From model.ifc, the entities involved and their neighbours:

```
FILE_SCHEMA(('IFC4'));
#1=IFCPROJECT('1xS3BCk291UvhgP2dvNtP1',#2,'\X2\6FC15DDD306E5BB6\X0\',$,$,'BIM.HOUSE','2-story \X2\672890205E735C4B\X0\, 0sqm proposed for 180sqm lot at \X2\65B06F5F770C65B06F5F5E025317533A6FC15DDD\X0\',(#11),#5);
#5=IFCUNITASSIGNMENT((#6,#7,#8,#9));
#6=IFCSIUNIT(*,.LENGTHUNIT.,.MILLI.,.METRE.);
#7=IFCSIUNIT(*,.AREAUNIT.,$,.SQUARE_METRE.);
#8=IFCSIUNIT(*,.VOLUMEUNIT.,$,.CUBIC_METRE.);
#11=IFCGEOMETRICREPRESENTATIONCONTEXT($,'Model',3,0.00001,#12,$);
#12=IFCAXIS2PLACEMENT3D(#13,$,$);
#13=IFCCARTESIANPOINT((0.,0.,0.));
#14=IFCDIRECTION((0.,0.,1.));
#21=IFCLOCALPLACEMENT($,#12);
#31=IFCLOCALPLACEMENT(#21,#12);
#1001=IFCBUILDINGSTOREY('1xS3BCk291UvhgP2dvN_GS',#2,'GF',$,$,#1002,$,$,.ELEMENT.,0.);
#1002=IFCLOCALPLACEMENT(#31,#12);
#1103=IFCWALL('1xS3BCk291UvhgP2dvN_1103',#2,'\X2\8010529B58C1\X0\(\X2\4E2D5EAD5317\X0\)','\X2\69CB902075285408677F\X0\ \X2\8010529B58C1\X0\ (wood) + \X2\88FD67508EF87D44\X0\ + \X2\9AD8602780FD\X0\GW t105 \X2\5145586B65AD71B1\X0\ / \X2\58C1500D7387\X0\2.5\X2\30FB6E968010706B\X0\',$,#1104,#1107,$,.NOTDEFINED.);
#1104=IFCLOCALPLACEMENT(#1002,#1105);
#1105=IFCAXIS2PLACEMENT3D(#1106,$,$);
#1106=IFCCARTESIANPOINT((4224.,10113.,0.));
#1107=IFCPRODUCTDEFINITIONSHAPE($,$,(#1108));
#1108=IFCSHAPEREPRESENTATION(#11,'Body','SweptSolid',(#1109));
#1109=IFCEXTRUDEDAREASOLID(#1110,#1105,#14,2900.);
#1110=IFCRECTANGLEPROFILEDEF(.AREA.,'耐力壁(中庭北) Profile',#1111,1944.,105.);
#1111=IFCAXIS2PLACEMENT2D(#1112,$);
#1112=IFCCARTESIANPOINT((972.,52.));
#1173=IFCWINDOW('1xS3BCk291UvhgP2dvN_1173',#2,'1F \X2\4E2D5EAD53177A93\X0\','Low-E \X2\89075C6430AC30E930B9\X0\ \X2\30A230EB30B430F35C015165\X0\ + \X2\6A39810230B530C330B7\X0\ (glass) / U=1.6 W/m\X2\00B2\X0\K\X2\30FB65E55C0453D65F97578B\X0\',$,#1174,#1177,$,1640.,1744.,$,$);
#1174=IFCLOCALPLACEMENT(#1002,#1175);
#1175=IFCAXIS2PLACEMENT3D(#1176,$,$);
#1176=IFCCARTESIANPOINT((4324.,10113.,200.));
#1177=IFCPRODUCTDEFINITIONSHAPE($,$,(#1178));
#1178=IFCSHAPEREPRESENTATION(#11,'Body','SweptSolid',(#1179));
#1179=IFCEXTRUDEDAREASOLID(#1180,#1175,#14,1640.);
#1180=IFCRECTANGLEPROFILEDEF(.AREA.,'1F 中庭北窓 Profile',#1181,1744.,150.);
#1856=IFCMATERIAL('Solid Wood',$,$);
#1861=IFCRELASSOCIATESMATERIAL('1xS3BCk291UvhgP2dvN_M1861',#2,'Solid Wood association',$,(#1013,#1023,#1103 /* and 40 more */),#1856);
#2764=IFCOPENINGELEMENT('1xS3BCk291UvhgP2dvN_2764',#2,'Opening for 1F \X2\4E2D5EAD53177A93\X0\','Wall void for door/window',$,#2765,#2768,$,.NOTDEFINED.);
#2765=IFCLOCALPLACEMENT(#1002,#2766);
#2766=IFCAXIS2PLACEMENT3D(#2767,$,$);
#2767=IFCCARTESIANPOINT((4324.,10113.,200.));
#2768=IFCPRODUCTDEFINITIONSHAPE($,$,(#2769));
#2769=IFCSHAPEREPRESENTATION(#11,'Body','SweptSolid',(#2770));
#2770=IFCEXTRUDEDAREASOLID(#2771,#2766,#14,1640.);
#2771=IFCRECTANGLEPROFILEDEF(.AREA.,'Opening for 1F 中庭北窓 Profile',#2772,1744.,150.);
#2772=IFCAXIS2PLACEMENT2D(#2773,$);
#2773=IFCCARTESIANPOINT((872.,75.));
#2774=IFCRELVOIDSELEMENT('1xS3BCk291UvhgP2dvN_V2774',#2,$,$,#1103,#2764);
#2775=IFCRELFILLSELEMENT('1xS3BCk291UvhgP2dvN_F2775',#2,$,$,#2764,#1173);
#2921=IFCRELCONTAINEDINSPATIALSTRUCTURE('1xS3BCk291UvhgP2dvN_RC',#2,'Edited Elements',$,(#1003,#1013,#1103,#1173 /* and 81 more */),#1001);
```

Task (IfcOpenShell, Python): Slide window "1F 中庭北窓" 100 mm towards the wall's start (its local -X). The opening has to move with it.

```python
import ifcopenshell
import ifcopenshell.api.geometry
import ifcopenshell.util.placement

model = ifcopenshell.open("model.ifc")

window = model.by_guid("1xS3BCk291UvhgP2dvN_1173")
opening = window.FillsVoids[0].RelatingOpeningElement
wall = opening.VoidsElements[0].RelatingBuildingElement

wall_matrix = ifcopenshell.util.placement.get_local_placement(wall.ObjectPlacement)
shift = wall_matrix[:3, 0] * -100.0
before = ifcopenshell.util.placement.get_local_placement(window.ObjectPlacement)[:3, 3].copy()

# The window is not placed relative to its opening, so move both.
for product in (opening, window):
    matrix = ifcopenshell.util.placement.get_local_placement(product.ObjectPlacement)
    matrix[:3, 3] += shift
    ifcopenshell.api.geometry.edit_object_placement(model, product=product, matrix=matrix, is_si=False)

after = ifcopenshell.util.placement.get_local_placement(window.ObjectPlacement)[:3, 3]
print("window moved by", (after - before).round(3) + 0.0)

model.write("model_rev.ifc")
```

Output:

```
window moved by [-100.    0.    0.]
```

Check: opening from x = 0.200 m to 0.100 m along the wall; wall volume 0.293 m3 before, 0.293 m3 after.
